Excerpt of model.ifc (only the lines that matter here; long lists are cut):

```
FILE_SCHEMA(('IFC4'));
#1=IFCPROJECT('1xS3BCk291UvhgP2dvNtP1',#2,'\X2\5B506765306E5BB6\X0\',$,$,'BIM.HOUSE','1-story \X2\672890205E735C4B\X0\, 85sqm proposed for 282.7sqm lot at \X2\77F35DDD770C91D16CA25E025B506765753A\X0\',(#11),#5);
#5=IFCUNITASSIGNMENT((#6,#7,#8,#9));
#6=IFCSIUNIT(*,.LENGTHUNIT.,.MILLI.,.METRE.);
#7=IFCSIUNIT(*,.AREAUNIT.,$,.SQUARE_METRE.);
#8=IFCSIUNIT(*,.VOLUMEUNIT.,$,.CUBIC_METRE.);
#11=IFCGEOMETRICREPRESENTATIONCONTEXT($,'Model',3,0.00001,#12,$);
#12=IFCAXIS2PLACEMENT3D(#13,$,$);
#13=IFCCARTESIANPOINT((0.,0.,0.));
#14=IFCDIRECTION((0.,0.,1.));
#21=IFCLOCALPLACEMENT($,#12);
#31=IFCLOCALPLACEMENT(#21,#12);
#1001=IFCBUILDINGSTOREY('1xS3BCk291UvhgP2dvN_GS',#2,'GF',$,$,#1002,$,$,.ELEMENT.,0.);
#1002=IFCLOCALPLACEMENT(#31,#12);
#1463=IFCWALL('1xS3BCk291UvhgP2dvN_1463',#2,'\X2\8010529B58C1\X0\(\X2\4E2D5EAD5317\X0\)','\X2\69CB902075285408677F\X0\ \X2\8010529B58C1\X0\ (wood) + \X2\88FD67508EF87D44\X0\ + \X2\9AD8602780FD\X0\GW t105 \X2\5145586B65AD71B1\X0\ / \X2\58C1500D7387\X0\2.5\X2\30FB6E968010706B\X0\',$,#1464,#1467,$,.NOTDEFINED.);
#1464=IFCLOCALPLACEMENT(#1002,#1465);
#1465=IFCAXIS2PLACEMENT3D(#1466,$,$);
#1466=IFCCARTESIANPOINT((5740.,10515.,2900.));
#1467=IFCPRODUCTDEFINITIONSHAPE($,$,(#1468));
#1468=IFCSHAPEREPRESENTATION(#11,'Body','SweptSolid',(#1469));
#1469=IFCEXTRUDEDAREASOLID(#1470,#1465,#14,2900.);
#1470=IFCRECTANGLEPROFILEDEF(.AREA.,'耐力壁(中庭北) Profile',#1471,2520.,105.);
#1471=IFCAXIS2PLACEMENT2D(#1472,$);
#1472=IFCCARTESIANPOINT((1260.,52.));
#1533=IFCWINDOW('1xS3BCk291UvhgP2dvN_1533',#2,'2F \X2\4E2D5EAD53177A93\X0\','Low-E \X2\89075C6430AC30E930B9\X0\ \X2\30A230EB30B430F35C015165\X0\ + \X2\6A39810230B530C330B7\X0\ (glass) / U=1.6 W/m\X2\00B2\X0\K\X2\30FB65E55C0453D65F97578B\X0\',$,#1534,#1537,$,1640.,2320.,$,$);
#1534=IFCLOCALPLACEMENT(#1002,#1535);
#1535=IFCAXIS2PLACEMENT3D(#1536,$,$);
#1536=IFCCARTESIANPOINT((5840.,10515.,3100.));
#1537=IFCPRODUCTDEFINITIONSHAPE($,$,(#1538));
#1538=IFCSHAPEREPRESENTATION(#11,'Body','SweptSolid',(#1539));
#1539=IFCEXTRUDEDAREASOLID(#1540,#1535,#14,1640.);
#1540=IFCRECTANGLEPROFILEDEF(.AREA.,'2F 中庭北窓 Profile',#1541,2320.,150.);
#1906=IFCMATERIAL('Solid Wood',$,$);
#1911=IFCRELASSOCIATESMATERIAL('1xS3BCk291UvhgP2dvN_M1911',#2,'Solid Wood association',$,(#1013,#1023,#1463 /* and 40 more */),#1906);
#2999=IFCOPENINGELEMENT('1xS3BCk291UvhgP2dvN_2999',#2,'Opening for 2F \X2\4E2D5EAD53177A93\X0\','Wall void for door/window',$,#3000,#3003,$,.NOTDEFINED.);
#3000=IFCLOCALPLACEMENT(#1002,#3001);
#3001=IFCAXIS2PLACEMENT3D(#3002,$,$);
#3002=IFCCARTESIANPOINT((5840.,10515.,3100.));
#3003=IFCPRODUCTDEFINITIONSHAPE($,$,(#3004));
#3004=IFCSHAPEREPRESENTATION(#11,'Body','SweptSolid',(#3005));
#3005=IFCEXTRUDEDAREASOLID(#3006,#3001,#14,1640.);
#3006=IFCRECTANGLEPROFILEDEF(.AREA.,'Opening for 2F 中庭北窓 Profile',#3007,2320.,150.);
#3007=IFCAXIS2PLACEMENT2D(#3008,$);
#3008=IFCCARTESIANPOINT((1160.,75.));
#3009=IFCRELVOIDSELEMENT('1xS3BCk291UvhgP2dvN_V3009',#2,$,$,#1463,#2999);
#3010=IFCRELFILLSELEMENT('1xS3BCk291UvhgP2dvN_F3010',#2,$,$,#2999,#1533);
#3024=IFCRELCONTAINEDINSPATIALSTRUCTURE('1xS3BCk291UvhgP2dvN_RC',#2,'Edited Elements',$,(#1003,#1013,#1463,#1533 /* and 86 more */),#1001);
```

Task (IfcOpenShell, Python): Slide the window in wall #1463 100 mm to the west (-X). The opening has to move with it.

```python
import ifcopenshell
import ifcopenshell.api.geometry
import ifcopenshell.util.placement
import ifcopenshell.util.unit

model = ifcopenshell.open("model.ifc")
unit_scale = ifcopenshell.util.unit.calculate_unit_scale(model)

window = model.by_guid("1xS3BCk291UvhgP2dvN_1533")
opening = window.FillsVoids[0].RelatingOpeningElement
wall = opening.VoidsElements[0].RelatingBuildingElement

wall_matrix = ifcopenshell.util.placement.get_local_placement(wall.ObjectPlacement)
shift = wall_matrix[:3, 0] * -0.1 / unit_scale
before = ifcopenshell.util.placement.get_local_placement(window.ObjectPlacement)[:3, 3].copy()

# The window is not placed relative to its opening, so move both.
for product in (opening, window):
    matrix = ifcopenshell.util.placement.get_local_placement(product.ObjectPlacement)
    matrix[:3, 3] += shift
    ifcopenshell.api.geometry.edit_object_placement(model, product=product, matrix=matrix, is_si=False)

after = ifcopenshell.util.placement.get_local_placement(window.ObjectPlacement)[:3, 3]
print("window moved by", (after - before).round(3) + 0.0)

model.write("model_rev.ifc")
```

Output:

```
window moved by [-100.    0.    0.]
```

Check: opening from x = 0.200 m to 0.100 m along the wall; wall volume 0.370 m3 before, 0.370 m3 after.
